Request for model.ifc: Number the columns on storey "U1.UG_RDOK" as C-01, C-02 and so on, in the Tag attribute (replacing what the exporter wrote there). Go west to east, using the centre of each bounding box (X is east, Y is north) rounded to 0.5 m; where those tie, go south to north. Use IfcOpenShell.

First a look at what the model holds.

```python
import ifcopenshell
import ifcopenshell.util.element
import ifcopenshell.util.placement

model = ifcopenshell.open("model.ifc")
print(model.schema)
storey = next(s for s in model.by_type("IfcBuildingStorey") if s.Name == "U1.UG_RDOK")
columns = [e for e in ifcopenshell.util.element.get_decomposition(storey) if e.is_a("IfcColumn")]
for e in sorted(columns, key=lambda e: e.id()):
    origin = ifcopenshell.util.placement.get_local_placement(e.ObjectPlacement)[:3, 3]
    print(e.id(), e.Tag, e.Name, origin.round(2) + 0.0, sep=" | ")
```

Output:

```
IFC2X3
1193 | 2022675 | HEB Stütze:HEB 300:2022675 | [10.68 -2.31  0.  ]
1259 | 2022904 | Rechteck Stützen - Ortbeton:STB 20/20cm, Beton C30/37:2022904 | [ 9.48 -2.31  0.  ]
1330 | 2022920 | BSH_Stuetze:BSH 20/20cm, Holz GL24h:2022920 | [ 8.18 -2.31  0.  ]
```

```python
import ifcopenshell
import ifcopenshell.geom
import ifcopenshell.util.element
import ifcopenshell.util.shape

model = ifcopenshell.open("model.ifc")
settings = ifcopenshell.geom.settings()
settings.set("use-world-coords", True)


def centre(element):
    shape = ifcopenshell.geom.create_shape(settings, element)
    return ifcopenshell.util.shape.get_bbox_centroid(shape.geometry)


storey = next(s for s in model.by_type("IfcBuildingStorey") if s.Name == "U1.UG_RDOK")
columns = [e for e in ifcopenshell.util.element.get_decomposition(storey) if e.is_a("IfcColumn")]

# Insertion points can sit at a corner or the storey origin, so sort by the geometry (in metres).
centres = {e: centre(e) for e in columns}
columns.sort(key=lambda e: (round(centres[e][0] / 0.5), centres[e][1]))

for i, e in enumerate(columns, start=1):
    number = f"C-{i:02d}"
    e.Tag = number
    print(e.id(), number)

model.write("model-out.ifc")
```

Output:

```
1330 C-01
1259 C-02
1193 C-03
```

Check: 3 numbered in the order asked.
